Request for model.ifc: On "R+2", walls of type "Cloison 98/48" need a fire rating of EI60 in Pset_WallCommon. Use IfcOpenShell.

First a look at what the model holds.

```python
import ifcopenshell
import ifcopenshell.util.element

model = ifcopenshell.open("model.ifc")
print(model.schema)
storey = next(s for s in model.by_type("IfcBuildingStorey") if s.Name == "R+2")
walls = [e for e in ifcopenshell.util.element.get_decomposition(storey) if e.is_a("IfcWall")]
seen = {}
for e in walls:
    element_type = ifcopenshell.util.element.get_type(e)
    key = (element_type.Name if element_type != e and element_type else None, ifcopenshell.util.element.get_pset(e, "Pset_WallCommon", "FireRating"))
    seen[key] = seen.get(key, 0) + 1
for (name, value), count in sorted(seen.items(), key=str):
    print(count, "x", name, "|", value)
```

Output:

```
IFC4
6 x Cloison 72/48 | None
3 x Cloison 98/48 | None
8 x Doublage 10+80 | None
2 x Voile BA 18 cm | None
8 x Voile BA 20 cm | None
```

```python
import ifcopenshell
import ifcopenshell.api.pset
import ifcopenshell.util.element

model = ifcopenshell.open("model.ifc")

storey = next(s for s in model.by_type("IfcBuildingStorey") if s.Name == "R+2")
walls = [e for e in ifcopenshell.util.element.get_decomposition(storey) if e.is_a("IfcWall")]

count = 0
for e in walls:
    element_type = ifcopenshell.util.element.get_type(e)
    if element_type in (None, e) or element_type.Name != "Cloison 98/48":
        continue
    # add_pset returns the element's existing set when there is one.
    pset = ifcopenshell.api.pset.add_pset(model, product=e, name="Pset_WallCommon")
    ifcopenshell.api.pset.edit_pset(model, pset=pset, properties={"FireRating": "EI60"})
    count += 1

print(count, "walls updated")

model.write("model_rev.ifc")
```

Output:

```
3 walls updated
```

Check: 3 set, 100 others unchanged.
